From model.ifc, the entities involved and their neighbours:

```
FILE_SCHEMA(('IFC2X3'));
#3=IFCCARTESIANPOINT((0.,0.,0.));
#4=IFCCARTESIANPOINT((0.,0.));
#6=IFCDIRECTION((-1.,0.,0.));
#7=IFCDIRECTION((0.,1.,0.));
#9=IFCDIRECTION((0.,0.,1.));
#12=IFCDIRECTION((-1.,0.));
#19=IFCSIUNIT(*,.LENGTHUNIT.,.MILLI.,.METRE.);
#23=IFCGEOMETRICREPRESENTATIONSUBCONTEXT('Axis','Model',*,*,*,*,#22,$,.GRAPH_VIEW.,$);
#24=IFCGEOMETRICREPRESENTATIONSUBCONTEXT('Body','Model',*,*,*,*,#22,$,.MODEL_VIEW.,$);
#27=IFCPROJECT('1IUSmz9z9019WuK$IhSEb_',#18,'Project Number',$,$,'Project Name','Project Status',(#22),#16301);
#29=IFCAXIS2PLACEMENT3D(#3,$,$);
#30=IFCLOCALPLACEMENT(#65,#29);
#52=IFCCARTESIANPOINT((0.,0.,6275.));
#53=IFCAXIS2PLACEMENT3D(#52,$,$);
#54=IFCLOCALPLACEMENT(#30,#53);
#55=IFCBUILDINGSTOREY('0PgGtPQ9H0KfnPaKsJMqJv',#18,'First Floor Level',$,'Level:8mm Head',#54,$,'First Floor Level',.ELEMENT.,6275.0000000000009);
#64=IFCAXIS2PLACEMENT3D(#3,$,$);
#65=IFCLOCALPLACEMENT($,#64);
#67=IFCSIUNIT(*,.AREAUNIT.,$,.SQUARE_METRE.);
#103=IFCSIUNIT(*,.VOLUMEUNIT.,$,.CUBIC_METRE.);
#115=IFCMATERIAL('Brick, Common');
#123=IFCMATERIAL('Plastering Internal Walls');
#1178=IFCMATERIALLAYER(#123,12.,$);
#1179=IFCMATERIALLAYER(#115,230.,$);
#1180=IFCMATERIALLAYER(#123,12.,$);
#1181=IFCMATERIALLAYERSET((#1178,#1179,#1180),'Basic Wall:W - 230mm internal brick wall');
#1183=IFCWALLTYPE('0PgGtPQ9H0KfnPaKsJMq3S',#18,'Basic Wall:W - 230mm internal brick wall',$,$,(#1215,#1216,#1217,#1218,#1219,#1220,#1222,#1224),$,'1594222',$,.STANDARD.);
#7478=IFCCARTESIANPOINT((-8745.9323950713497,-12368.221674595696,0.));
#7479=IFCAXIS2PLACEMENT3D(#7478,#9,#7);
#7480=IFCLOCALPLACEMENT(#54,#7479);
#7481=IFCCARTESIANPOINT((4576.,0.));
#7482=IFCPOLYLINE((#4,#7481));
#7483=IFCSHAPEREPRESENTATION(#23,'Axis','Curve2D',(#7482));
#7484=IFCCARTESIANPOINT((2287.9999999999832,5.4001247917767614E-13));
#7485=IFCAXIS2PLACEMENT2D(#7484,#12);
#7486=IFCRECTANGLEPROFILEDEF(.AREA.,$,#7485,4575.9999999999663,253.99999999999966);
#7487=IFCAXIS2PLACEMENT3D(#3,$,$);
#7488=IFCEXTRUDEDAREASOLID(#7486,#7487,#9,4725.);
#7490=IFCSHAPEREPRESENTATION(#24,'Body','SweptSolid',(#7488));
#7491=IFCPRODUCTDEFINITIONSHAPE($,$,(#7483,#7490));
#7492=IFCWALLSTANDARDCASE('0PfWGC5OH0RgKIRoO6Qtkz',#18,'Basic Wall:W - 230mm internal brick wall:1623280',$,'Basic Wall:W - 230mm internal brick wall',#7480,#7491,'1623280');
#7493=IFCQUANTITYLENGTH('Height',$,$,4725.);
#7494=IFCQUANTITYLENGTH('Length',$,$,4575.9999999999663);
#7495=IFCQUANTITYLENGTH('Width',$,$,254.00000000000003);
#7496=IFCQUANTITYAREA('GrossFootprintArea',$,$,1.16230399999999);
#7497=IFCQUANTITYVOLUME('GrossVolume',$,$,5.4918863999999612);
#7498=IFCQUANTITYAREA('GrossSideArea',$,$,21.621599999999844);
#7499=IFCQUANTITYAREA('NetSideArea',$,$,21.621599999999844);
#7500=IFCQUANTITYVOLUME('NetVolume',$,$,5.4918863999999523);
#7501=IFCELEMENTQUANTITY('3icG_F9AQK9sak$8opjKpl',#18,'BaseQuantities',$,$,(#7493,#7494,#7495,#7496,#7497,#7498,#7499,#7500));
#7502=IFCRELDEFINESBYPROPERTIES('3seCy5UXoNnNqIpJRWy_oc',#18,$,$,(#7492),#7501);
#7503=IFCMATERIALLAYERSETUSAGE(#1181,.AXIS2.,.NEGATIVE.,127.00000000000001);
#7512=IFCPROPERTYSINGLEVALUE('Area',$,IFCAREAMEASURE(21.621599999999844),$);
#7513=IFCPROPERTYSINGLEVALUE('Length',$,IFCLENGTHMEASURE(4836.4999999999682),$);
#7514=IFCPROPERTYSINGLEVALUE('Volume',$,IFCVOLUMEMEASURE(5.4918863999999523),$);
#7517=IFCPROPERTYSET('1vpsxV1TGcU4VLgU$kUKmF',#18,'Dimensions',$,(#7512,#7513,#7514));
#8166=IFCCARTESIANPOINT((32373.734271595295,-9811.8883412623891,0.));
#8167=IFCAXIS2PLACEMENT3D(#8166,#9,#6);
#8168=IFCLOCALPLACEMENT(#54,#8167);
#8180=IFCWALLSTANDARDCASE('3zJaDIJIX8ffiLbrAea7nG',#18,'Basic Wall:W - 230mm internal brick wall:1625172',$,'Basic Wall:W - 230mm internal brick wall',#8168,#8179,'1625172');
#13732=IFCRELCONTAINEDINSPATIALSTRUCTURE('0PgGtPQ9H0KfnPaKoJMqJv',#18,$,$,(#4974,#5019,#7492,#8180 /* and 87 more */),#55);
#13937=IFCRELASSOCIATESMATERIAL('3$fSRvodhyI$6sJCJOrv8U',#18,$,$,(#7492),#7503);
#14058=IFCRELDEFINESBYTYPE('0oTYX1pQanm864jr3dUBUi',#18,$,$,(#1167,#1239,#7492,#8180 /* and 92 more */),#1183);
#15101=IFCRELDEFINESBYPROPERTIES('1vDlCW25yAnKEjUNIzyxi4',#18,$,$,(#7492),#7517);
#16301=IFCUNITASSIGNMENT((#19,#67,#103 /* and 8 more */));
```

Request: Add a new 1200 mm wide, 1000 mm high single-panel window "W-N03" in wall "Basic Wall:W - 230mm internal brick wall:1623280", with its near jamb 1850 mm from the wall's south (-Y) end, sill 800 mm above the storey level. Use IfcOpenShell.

```python
import numpy as np
import ifcopenshell
import ifcopenshell.api.feature
import ifcopenshell.api.geometry
import ifcopenshell.api.pset
import ifcopenshell.api.root
import ifcopenshell.api.spatial
import ifcopenshell.api.type
import ifcopenshell.geom
import ifcopenshell.util.element
import ifcopenshell.util.placement
import ifcopenshell.util.representation
import ifcopenshell.util.shape
import ifcopenshell.util.unit

model = ifcopenshell.open("model.ifc")
unit_scale = ifcopenshell.util.unit.calculate_unit_scale(model)
area_scale = ifcopenshell.util.unit.calculate_unit_scale(model, "AREAUNIT")
volume_scale = ifcopenshell.util.unit.calculate_unit_scale(model, "VOLUMEUNIT")
settings = ifcopenshell.geom.settings()


def volume(element):
    """Net volume in cubic metres, openings subtracted."""
    shape = ifcopenshell.geom.create_shape(settings, element)
    return ifcopenshell.util.shape.get_volume(shape.geometry)


wall = model.by_guid("0PfWGC5OH0RgKIRoO6Qtkz")
storey = ifcopenshell.util.element.get_container(wall, ifc_class="IfcBuildingStorey")
context = ifcopenshell.util.representation.get_context(model, "Model", "Body", "MODEL_VIEW")
before = volume(wall)

width, height, from_end, sill = 1.2, 1, 1.85, 0.8  # metres

# The wall runs along its own X axis, and the end named is its -X end.
wall_shape = ifcopenshell.geom.create_shape(settings, wall)
x, y, z = ifcopenshell.util.shape.get_vertices(wall_shape.geometry).T
start = x.min() + from_end
face, thickness = float(y.min()), float(y.max() - y.min())
wall_matrix = ifcopenshell.util.placement.get_local_placement(wall.ObjectPlacement)
level = ifcopenshell.util.placement.get_local_placement(storey.ObjectPlacement)[2, 3]


def in_wall(x, y):
    """Placement at x, y metres in the wall's axes, at sill height."""
    matrix = wall_matrix.copy()
    matrix[:, 3] = wall_matrix @ np.array([x / unit_scale, y / unit_scale, 0.0, 1.0])
    matrix[2, 3] = level + sill / unit_scale
    return matrix


# Opening: a box that overshoots both wall faces by 50 mm.
opening = ifcopenshell.api.root.create_entity(model, ifc_class="IfcOpeningElement")
box = ifcopenshell.api.geometry.add_wall_representation(
    model, context=context, length=width, height=height, thickness=thickness + 0.1
)
ifcopenshell.api.geometry.assign_representation(model, product=opening, representation=box)
ifcopenshell.api.geometry.edit_object_placement(model, product=opening, matrix=in_wall(start, face - 0.05), is_si=False)
ifcopenshell.api.feature.add_feature(model, feature=opening, element=wall)

window = ifcopenshell.api.root.create_entity(model, ifc_class="IfcWindow", name="W-N03")
window.OverallWidth, window.OverallHeight = width / unit_scale, height / unit_scale
body = ifcopenshell.api.geometry.add_window_representation(
    model,
    context=context,
    overall_width=window.OverallWidth,
    overall_height=window.OverallHeight,
    partition_type="SINGLE_PANEL",
)
ifcopenshell.api.geometry.assign_representation(model, product=window, representation=body)
ifcopenshell.api.spatial.assign_container(model, products=[window], relating_structure=storey)
fills = ifcopenshell.api.feature.add_filling(model, opening=opening, element=window)
fills.OwnerHistory = window.OwnerHistory  # required in IFC2X3

# IFC2X3 keeps the operation on the window style.
style = ifcopenshell.api.root.create_entity(model, ifc_class="IfcWindowStyle", name="W-N03")
style.OperationType, style.ConstructionType = "SINGLE_PANEL", "NOTDEFINED"
style.ParameterTakesPrecedence = style.Sizeable = False
ifcopenshell.api.type.assign_type(model, related_objects=[window], relating_type=style)

# Centre the window in the wall's thickness.
ifcopenshell.api.geometry.edit_object_placement(model, product=window, matrix=in_wall(start, face), is_si=False)
window_shape = ifcopenshell.geom.create_shape(settings, window)
depth = ifcopenshell.util.shape.get_vertices(window_shape.geometry)[:, 1]
offset = face + thickness / 2 - (depth.min() + depth.max()) / 2
ifcopenshell.api.geometry.edit_object_placement(model, product=window, matrix=in_wall(start, offset), is_si=False)

after = volume(wall)

# Update the wall's stored quantities.
qto = model.by_id(ifcopenshell.util.element.get_pset(wall, "BaseQuantities", should_inherit=False)["id"])
ifcopenshell.api.pset.edit_qto(model, qto=qto, properties={
    "NetSideArea": after / thickness / area_scale,
    "NetVolume": after / volume_scale,
})
pset = model.by_id(ifcopenshell.util.element.get_pset(wall, "Dimensions", should_inherit=False)["id"])
ifcopenshell.api.pset.edit_pset(model, pset=pset, properties={
    "Area": model.create_entity("IfcAreaMeasure", after / thickness / area_scale),
    "Volume": model.create_entity("IfcVolumeMeasure", after / volume_scale),
})

print(f"wall volume {before:.3f} -> {after:.3f} m3")

model.write("model_rev.ifc")
```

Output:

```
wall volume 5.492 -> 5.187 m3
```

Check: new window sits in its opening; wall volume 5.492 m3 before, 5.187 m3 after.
